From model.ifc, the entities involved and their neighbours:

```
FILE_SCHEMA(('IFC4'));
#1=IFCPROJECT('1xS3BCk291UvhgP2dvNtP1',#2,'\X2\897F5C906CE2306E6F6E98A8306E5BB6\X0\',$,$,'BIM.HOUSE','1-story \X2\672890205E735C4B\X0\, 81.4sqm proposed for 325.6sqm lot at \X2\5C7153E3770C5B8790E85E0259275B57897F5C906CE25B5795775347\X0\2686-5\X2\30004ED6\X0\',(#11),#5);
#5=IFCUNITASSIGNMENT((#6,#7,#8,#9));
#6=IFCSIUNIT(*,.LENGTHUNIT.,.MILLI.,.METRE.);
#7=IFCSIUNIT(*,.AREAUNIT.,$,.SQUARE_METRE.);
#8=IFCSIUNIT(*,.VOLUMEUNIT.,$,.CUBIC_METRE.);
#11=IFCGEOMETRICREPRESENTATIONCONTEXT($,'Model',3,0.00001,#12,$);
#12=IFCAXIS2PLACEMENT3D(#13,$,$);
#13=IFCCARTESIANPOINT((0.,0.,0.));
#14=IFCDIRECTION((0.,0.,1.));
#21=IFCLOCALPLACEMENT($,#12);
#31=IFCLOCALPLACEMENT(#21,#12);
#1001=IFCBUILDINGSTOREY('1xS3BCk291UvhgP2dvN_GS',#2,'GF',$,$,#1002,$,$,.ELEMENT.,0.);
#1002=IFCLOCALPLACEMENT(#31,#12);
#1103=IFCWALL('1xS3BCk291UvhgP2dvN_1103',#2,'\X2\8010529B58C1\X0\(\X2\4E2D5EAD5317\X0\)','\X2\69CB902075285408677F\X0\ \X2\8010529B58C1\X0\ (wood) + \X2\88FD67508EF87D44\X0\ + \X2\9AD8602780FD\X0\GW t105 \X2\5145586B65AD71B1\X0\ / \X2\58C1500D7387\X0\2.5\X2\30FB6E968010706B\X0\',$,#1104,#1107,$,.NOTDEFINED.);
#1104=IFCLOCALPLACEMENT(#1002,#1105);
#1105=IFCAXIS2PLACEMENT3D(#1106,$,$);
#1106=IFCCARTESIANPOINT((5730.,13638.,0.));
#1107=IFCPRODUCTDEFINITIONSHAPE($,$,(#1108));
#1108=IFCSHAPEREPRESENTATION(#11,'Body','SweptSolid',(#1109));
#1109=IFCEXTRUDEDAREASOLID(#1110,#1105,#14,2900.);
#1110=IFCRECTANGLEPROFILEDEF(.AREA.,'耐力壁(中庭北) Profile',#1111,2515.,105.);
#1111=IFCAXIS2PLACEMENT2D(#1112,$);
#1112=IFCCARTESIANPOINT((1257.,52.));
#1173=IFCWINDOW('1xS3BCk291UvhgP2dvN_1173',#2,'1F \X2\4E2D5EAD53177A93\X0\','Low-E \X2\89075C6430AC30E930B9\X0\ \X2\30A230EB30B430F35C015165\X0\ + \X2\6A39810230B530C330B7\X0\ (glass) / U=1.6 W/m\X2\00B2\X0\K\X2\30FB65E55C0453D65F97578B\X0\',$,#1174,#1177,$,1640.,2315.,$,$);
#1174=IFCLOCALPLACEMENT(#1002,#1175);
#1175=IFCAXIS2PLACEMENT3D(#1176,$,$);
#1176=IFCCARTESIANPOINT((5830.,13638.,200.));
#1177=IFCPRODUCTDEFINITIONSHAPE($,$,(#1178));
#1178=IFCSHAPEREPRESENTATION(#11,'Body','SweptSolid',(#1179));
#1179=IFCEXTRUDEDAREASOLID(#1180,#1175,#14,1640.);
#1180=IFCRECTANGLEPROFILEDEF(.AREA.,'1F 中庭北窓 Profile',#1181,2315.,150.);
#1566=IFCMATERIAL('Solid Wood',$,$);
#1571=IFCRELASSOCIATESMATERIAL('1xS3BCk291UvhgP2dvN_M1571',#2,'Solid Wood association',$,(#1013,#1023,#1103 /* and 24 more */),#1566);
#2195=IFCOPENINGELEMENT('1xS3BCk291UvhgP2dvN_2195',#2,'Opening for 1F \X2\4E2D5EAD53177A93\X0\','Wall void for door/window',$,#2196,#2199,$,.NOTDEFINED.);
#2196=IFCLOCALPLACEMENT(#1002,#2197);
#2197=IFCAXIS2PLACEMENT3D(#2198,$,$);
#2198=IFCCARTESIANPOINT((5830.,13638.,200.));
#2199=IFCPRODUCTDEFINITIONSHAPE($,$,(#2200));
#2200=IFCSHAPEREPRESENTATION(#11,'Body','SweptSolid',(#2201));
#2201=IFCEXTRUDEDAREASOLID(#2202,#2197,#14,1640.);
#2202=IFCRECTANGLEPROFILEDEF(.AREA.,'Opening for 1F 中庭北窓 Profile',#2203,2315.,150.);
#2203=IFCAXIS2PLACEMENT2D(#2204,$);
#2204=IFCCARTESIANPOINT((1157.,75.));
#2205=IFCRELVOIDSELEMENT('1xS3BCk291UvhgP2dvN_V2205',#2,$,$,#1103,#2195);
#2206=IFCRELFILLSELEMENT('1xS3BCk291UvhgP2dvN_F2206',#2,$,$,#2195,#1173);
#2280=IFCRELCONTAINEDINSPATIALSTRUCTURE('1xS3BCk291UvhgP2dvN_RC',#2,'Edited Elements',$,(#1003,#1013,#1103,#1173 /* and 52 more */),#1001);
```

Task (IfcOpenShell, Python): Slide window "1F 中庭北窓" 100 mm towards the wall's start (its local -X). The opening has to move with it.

```python
import ifcopenshell
import ifcopenshell.api.geometry
import ifcopenshell.util.placement
import ifcopenshell.util.unit

model = ifcopenshell.open("model.ifc")
unit_scale = ifcopenshell.util.unit.calculate_unit_scale(model)

window = model.by_id(1173)
opening = window.FillsVoids[0].RelatingOpeningElement
wall = opening.VoidsElements[0].RelatingBuildingElement

wall_matrix = ifcopenshell.util.placement.get_local_placement(wall.ObjectPlacement)
shift = wall_matrix[:3, 0] * -0.1 / unit_scale
before = ifcopenshell.util.placement.get_local_placement(window.ObjectPlacement)[:3, 3].copy()

# The window is not placed relative to its opening, so move both.
for product in (opening, window):
    matrix = ifcopenshell.util.placement.get_local_placement(product.ObjectPlacement)
    matrix[:3, 3] += shift
    ifcopenshell.api.geometry.edit_object_placement(model, product=product, matrix=matrix, is_si=False)

after = ifcopenshell.util.placement.get_local_placement(window.ObjectPlacement)[:3, 3]
print("window moved by", (after - before).round(3) + 0.0)

model.write("model-out.ifc")
```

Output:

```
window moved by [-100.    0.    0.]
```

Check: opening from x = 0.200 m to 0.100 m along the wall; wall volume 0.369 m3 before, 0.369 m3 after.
